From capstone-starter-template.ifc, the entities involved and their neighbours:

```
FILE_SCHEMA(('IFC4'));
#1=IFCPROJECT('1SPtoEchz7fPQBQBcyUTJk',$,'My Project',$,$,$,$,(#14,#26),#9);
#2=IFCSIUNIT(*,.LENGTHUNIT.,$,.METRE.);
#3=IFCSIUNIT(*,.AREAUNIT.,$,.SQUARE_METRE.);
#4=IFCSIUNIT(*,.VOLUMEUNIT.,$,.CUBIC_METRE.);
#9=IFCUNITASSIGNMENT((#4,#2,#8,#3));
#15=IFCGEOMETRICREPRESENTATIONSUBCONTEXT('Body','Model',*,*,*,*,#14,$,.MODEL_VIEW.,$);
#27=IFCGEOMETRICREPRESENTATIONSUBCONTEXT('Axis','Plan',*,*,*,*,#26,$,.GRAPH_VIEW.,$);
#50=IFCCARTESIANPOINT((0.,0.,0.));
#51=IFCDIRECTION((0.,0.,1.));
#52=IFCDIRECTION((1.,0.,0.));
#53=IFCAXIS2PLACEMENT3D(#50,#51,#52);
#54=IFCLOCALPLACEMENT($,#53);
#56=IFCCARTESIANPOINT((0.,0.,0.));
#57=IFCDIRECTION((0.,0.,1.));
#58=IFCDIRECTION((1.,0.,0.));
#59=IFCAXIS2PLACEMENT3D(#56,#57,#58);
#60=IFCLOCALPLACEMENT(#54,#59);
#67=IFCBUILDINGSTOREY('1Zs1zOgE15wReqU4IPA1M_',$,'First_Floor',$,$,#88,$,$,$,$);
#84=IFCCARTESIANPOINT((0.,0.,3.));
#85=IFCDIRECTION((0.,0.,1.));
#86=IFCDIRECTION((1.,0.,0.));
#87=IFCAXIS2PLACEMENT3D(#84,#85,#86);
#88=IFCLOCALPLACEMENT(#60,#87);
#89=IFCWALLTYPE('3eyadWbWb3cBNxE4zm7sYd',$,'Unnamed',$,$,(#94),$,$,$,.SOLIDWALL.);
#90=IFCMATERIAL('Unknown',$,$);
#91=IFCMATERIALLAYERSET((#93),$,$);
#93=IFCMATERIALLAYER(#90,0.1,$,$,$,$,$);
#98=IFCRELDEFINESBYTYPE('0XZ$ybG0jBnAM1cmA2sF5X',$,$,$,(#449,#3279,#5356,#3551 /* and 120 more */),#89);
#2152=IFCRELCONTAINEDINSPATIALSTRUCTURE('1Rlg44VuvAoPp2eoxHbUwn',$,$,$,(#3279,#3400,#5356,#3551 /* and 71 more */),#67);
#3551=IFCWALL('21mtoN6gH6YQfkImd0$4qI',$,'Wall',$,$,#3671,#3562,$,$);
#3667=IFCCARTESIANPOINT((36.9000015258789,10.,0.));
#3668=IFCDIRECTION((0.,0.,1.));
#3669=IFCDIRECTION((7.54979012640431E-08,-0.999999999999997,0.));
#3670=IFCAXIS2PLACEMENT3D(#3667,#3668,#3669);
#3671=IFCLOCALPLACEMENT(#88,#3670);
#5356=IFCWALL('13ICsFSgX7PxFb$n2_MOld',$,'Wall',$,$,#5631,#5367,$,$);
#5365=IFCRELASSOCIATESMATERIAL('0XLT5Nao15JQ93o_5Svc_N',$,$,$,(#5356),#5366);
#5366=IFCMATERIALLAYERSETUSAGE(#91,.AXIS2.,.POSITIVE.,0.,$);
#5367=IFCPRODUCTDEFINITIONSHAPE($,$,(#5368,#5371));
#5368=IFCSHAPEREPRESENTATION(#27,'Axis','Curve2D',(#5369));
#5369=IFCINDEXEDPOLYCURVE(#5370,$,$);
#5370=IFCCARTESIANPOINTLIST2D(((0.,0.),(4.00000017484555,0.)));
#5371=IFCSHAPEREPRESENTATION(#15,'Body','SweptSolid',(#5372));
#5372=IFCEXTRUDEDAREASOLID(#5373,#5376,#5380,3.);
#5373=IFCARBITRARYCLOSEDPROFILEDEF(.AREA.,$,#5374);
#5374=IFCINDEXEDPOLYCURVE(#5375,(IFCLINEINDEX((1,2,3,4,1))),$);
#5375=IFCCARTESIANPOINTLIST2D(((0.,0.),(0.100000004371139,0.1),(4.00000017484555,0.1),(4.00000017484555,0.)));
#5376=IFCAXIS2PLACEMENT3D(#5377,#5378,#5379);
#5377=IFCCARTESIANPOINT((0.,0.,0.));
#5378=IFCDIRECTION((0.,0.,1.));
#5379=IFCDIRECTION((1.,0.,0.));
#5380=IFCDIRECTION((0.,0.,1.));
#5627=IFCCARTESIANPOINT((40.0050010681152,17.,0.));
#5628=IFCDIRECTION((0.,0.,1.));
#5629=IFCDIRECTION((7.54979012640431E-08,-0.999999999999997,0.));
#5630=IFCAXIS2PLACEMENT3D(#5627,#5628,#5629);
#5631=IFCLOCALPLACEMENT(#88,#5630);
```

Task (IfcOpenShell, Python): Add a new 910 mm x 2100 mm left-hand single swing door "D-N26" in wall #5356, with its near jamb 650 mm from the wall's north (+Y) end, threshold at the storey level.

```python
import numpy as np
import ifcopenshell
import ifcopenshell.api.feature
import ifcopenshell.api.geometry
import ifcopenshell.api.root
import ifcopenshell.api.spatial
import ifcopenshell.geom
import ifcopenshell.util.element
import ifcopenshell.util.placement
import ifcopenshell.util.representation
import ifcopenshell.util.shape
import ifcopenshell.util.unit

model = ifcopenshell.open("capstone-starter-template.ifc")
unit_scale = ifcopenshell.util.unit.calculate_unit_scale(model)
settings = ifcopenshell.geom.settings()


def volume(element):
    """Net volume in cubic metres, openings subtracted."""
    shape = ifcopenshell.geom.create_shape(settings, element)
    return ifcopenshell.util.shape.get_volume(shape.geometry)


wall = model.by_id(5356)
storey = ifcopenshell.util.element.get_container(wall, ifc_class="IfcBuildingStorey")
context = ifcopenshell.util.representation.get_context(model, "Model", "Body", "MODEL_VIEW")
before = volume(wall)

width, height, from_end, sill = 0.91, 2.1, 0.65, 0.0  # metres

# The wall runs along its own X axis, and the end named is its -X end.
wall_shape = ifcopenshell.geom.create_shape(settings, wall)
x, y, z = ifcopenshell.util.shape.get_vertices(wall_shape.geometry).T
start = x.min() + from_end
face, thickness = float(y.min()), float(y.max() - y.min())
wall_matrix = ifcopenshell.util.placement.get_local_placement(wall.ObjectPlacement)
level = ifcopenshell.util.placement.get_local_placement(storey.ObjectPlacement)[2, 3]


def in_wall(x, y):
    """Placement at x, y metres in the wall's axes, at sill height."""
    matrix = wall_matrix.copy()
    matrix[:, 3] = wall_matrix @ np.array([x / unit_scale, y / unit_scale, 0.0, 1.0])
    matrix[2, 3] = level + sill / unit_scale
    return matrix


# Opening: a box that overshoots both wall faces by 50 mm.
opening = ifcopenshell.api.root.create_entity(model, ifc_class="IfcOpeningElement", predefined_type="OPENING")
box = ifcopenshell.api.geometry.add_wall_representation(
    model, context=context, length=width, height=height, thickness=thickness + 0.1
)
ifcopenshell.api.geometry.assign_representation(model, product=opening, representation=box)
ifcopenshell.api.geometry.edit_object_placement(model, product=opening, matrix=in_wall(start, face - 0.05), is_si=False)
ifcopenshell.api.feature.add_feature(model, feature=opening, element=wall)

door = ifcopenshell.api.root.create_entity(model, ifc_class="IfcDoor", name="D-N26", predefined_type="DOOR")
door.OverallWidth, door.OverallHeight = width / unit_scale, height / unit_scale
door.OperationType = "SINGLE_SWING_LEFT"
body = ifcopenshell.api.geometry.add_door_representation(
    model,
    context=context,
    overall_width=door.OverallWidth,
    overall_height=door.OverallHeight,
    operation_type="SINGLE_SWING_LEFT",
    lining_properties={"LiningDepth": thickness / unit_scale, "ThresholdDepth": thickness / unit_scale},
)
ifcopenshell.api.geometry.assign_representation(model, product=door, representation=body)
ifcopenshell.api.spatial.assign_container(model, products=[door], relating_structure=storey)
ifcopenshell.api.feature.add_filling(model, opening=opening, element=door)

# The lining spans the wall, so the door starts at the wall face.
ifcopenshell.api.geometry.edit_object_placement(model, product=door, matrix=in_wall(start, face), is_si=False)

after = volume(wall)

print(f"wall volume {before:.3f} -> {after:.3f} m3")

model.write("capstone-starter-template_edited.ifc")
```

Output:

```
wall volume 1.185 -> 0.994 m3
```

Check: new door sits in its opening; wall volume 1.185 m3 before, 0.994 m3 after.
